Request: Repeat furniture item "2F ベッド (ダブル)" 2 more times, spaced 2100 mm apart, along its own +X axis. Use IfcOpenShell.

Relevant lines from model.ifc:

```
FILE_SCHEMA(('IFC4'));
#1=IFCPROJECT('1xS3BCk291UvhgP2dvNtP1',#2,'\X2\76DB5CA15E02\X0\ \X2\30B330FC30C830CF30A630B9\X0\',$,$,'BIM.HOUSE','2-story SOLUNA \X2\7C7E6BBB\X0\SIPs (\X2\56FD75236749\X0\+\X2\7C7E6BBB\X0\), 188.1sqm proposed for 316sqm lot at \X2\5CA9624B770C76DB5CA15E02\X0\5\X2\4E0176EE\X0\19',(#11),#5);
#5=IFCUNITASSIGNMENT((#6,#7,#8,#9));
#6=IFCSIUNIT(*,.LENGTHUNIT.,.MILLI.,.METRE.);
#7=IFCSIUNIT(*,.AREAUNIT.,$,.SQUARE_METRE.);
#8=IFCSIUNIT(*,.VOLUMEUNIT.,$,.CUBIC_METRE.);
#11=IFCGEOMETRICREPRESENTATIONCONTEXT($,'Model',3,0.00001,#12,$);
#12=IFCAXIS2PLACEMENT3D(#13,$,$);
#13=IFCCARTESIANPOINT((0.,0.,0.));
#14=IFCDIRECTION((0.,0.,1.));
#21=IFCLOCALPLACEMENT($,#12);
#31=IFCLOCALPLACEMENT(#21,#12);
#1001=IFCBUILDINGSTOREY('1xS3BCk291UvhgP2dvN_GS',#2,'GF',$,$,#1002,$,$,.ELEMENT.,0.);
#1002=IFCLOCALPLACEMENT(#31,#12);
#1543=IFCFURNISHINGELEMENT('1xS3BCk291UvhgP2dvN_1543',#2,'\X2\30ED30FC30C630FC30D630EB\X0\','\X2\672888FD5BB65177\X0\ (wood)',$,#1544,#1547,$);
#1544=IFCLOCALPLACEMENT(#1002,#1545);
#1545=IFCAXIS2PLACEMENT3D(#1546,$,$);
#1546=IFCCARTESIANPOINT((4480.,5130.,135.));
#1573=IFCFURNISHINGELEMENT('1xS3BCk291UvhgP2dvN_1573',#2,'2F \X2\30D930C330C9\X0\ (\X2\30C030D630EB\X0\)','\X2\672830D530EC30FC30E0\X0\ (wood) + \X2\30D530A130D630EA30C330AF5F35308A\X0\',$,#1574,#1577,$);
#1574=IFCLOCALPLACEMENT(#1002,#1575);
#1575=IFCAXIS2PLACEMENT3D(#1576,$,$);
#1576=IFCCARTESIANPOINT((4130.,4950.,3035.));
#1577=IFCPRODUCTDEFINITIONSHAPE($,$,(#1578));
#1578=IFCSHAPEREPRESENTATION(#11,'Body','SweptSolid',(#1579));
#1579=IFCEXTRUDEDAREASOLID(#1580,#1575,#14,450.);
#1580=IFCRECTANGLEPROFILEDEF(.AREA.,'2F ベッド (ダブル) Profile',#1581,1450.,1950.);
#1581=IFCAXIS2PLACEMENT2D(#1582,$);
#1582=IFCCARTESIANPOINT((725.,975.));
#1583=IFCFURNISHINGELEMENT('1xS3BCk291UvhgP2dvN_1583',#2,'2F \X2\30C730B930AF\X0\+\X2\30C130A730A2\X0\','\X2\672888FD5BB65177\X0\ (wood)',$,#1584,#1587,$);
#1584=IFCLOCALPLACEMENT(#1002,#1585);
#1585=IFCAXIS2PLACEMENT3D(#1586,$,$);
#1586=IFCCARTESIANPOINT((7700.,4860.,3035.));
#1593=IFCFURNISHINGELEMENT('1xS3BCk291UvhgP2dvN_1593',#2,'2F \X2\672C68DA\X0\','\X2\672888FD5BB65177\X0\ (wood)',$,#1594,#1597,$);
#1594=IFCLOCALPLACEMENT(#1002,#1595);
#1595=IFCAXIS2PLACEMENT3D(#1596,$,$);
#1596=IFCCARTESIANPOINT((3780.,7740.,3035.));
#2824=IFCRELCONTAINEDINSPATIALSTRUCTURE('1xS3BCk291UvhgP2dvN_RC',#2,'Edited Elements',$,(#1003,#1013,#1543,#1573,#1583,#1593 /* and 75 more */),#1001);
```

```python
import ifcopenshell
import ifcopenshell.api.geometry
import ifcopenshell.api.root
import ifcopenshell.util.element
import ifcopenshell.util.placement
import ifcopenshell.util.unit

model = ifcopenshell.open("model.ifc")
unit_scale = ifcopenshell.util.unit.calculate_unit_scale(model)


def reuse_history(source, copy):
    """copy_class also copies each property set's owner history, people and application; keep the originals."""
    for rel in copy.IsDefinedBy:
        if rel.is_a("IfcRelDefinesByProperties") and (history := rel.RelatingPropertyDefinition.OwnerHistory):
            rel.RelatingPropertyDefinition.OwnerHistory = source.OwnerHistory
            ifcopenshell.util.element.remove_deep2(model, history)


source = model.by_guid("1xS3BCk291UvhgP2dvN_1573")
base = ifcopenshell.util.placement.get_local_placement(source.ObjectPlacement)
step = base[:3, 0] * 2.1 / unit_scale

for i in range(1, 3):
    copy = ifcopenshell.api.root.copy_class(model, product=source)
    copy.Representation = ifcopenshell.util.element.copy_deep(
        model, source.Representation, exclude=["IfcGeometricRepresentationContext", "IfcRepresentationMap"]
    )
    reuse_history(source, copy)
    matrix = base.copy()
    matrix[:3, 3] += i * step
    print("added at", matrix[:3, 3].round(3) + 0.0)
    ifcopenshell.api.geometry.edit_object_placement(model, product=copy, matrix=matrix, is_si=False)

model.write("model_rev.ifc")
```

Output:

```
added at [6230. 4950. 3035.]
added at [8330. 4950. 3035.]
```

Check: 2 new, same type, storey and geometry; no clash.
